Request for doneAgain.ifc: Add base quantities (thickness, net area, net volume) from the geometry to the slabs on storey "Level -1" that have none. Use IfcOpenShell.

First a look at what the model holds.

```python
import ifcopenshell
import ifcopenshell.util.element
import ifcopenshell.util.unit

model = ifcopenshell.open("doneAgain.ifc")
print(model.schema)
for unit_type in ("LENGTHUNIT", "AREAUNIT", "VOLUMEUNIT"):
    print(unit_type, ifcopenshell.util.unit.calculate_unit_scale(model, unit_type))
storey = next(s for s in model.by_type("IfcBuildingStorey") if s.Name == "Level -1")
slabs = [e for e in ifcopenshell.util.element.get_decomposition(storey) if e.is_a("IfcSlab")]
for e in sorted(slabs, key=lambda e: e.id()):
    print(e.id(), e.is_a(), e.Name, list(ifcopenshell.util.element.get_psets(e, qtos_only=True)), sep=" | ")
```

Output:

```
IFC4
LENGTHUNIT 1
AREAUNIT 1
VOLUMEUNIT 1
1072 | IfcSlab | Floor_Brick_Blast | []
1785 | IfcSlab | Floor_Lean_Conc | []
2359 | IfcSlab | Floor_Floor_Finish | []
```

```python
import ifcopenshell
import ifcopenshell.api.pset
import ifcopenshell.geom
import ifcopenshell.util.element
import ifcopenshell.util.shape
import ifcopenshell.util.unit

model = ifcopenshell.open("doneAgain.ifc")
unit_scale = ifcopenshell.util.unit.calculate_unit_scale(model)
area_scale = ifcopenshell.util.unit.calculate_unit_scale(model, "AREAUNIT")
volume_scale = ifcopenshell.util.unit.calculate_unit_scale(model, "VOLUMEUNIT")
settings = ifcopenshell.geom.settings()

storey = next(s for s in model.by_type("IfcBuildingStorey") if s.Name == "Level -1")
slabs = [e for e in ifcopenshell.util.element.get_decomposition(storey) if e.is_a("IfcSlab")]

for e in sorted(slabs, key=lambda e: e.id()):
    if ifcopenshell.util.element.get_psets(e, qtos_only=True, should_inherit=False):
        continue
    # Geometry comes back in metres, in the element's own axes.
    shape = ifcopenshell.geom.create_shape(settings, e)
    values = {
        "Width": ifcopenshell.util.shape.get_z(shape.geometry) / unit_scale,
        "NetArea": ifcopenshell.util.shape.get_footprint_area(shape.geometry) / area_scale,
        "NetVolume": ifcopenshell.util.shape.get_volume(shape.geometry) / volume_scale,
    }
    qto = ifcopenshell.api.pset.add_qto(model, product=e, name="Qto_SlabBaseQuantities")
    ifcopenshell.api.pset.edit_qto(model, qto=qto, properties=values)
    print(e.id(), {k: round(v, 3) for k, v in values.items()})

model.write("doneAgain_updated.ifc")
```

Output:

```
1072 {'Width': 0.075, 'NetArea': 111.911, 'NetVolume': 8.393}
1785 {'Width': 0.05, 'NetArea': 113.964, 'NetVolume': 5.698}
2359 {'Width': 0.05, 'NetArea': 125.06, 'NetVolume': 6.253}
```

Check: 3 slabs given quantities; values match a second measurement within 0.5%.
